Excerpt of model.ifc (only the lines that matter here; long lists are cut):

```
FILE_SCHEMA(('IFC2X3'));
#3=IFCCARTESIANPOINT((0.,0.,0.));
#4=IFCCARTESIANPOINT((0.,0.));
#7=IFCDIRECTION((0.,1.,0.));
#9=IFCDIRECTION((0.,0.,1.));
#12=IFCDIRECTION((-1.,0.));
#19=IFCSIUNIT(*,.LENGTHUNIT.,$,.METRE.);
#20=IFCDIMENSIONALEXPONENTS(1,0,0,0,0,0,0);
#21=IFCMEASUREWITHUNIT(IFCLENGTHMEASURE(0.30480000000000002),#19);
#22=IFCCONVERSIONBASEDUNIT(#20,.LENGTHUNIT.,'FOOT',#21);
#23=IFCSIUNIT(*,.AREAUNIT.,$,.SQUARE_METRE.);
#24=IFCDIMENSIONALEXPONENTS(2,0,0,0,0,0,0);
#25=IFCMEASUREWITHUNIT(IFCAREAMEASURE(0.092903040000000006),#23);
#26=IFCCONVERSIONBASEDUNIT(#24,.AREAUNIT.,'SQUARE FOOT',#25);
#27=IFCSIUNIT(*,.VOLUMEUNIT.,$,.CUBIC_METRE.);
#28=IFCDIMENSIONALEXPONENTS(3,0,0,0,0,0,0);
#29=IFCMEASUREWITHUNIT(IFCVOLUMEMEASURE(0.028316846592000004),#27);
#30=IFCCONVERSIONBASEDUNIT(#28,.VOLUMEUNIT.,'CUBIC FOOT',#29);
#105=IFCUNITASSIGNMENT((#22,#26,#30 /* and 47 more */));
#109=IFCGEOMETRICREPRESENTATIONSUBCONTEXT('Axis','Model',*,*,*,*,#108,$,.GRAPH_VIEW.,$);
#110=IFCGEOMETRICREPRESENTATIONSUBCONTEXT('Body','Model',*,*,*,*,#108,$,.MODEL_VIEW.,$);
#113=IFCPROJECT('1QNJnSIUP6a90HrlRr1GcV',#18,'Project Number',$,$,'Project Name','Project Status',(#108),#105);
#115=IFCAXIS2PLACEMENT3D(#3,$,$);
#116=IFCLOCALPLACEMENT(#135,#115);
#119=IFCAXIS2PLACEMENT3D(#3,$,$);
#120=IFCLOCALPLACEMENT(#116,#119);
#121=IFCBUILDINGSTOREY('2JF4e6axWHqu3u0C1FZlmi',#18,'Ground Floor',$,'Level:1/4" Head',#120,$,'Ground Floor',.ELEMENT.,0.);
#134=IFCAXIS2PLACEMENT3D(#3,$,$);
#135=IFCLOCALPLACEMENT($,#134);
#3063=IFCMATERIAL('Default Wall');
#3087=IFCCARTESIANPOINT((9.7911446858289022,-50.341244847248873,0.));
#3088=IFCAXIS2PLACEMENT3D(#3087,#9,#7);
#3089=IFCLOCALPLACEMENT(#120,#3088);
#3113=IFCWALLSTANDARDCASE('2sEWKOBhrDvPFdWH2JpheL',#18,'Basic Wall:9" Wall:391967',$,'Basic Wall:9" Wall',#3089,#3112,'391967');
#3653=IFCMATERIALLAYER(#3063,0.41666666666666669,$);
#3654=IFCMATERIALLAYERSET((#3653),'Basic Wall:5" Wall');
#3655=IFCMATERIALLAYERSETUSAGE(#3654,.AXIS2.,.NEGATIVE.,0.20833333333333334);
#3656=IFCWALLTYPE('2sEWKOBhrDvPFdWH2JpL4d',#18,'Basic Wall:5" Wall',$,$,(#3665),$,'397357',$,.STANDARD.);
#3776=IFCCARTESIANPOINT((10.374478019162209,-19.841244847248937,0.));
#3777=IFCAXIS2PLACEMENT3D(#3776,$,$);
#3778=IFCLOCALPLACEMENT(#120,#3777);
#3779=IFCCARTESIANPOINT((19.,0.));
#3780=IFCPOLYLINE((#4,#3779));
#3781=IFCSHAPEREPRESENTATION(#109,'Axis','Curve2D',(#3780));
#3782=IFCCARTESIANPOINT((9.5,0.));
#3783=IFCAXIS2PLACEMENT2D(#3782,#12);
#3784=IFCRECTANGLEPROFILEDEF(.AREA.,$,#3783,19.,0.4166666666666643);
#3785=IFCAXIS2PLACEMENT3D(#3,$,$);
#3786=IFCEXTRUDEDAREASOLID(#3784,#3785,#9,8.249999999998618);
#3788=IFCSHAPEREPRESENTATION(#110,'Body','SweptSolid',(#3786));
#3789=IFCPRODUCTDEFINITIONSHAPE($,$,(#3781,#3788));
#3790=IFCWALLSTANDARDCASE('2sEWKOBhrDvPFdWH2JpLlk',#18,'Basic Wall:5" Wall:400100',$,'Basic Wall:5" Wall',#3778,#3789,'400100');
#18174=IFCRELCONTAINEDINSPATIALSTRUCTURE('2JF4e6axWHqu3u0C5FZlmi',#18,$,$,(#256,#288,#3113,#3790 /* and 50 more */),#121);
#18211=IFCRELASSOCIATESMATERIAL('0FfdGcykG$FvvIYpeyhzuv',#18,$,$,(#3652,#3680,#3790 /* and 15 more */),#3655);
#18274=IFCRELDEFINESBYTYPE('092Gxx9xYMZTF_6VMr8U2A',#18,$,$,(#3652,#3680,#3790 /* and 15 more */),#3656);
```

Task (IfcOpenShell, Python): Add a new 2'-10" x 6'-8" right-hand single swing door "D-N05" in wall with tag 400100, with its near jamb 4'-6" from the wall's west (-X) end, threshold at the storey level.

```python
import numpy as np
import ifcopenshell
import ifcopenshell.api.feature
import ifcopenshell.api.geometry
import ifcopenshell.api.root
import ifcopenshell.api.spatial
import ifcopenshell.api.type
import ifcopenshell.geom
import ifcopenshell.util.element
import ifcopenshell.util.placement
import ifcopenshell.util.representation
import ifcopenshell.util.shape
import ifcopenshell.util.unit

model = ifcopenshell.open("model.ifc")
unit_scale = ifcopenshell.util.unit.calculate_unit_scale(model)
settings = ifcopenshell.geom.settings()


def volume(element):
    """Net volume in cubic metres, openings subtracted."""
    shape = ifcopenshell.geom.create_shape(settings, element)
    return ifcopenshell.util.shape.get_volume(shape.geometry)


wall = model.by_guid("2sEWKOBhrDvPFdWH2JpLlk")
storey = ifcopenshell.util.element.get_container(wall, ifc_class="IfcBuildingStorey")
context = ifcopenshell.util.representation.get_context(model, "Model", "Body", "MODEL_VIEW")
before = volume(wall)

width, height, from_end, sill = 0.8636, 2.032, 1.3716, 0.0  # metres

# The wall runs along its own X axis, and the end named is its -X end.
wall_shape = ifcopenshell.geom.create_shape(settings, wall)
x, y, z = ifcopenshell.util.shape.get_vertices(wall_shape.geometry).T
start = x.min() + from_end
face, thickness = float(y.min()), float(y.max() - y.min())
wall_matrix = ifcopenshell.util.placement.get_local_placement(wall.ObjectPlacement)
level = ifcopenshell.util.placement.get_local_placement(storey.ObjectPlacement)[2, 3]


def in_wall(x, y):
    """Placement at x, y metres in the wall's axes, at sill height."""
    matrix = wall_matrix.copy()
    matrix[:, 3] = wall_matrix @ np.array([x / unit_scale, y / unit_scale, 0.0, 1.0])
    matrix[2, 3] = level + sill / unit_scale
    return matrix


# Opening: a box that overshoots both wall faces by 50 mm.
opening = ifcopenshell.api.root.create_entity(model, ifc_class="IfcOpeningElement")
box = ifcopenshell.api.geometry.add_wall_representation(
    model, context=context, length=width, height=height, thickness=thickness + 0.1
)
ifcopenshell.api.geometry.assign_representation(model, product=opening, representation=box)
ifcopenshell.api.geometry.edit_object_placement(model, product=opening, matrix=in_wall(start, face - 0.05), is_si=False)
ifcopenshell.api.feature.add_feature(model, feature=opening, element=wall)

door = ifcopenshell.api.root.create_entity(model, ifc_class="IfcDoor", name="D-N05")
door.OverallWidth, door.OverallHeight = width / unit_scale, height / unit_scale
body = ifcopenshell.api.geometry.add_door_representation(
    model,
    context=context,
    overall_width=door.OverallWidth,
    overall_height=door.OverallHeight,
    operation_type="SINGLE_SWING_RIGHT",
    lining_properties={"LiningDepth": thickness / unit_scale, "ThresholdDepth": thickness / unit_scale},
)
ifcopenshell.api.geometry.assign_representation(model, product=door, representation=body)
ifcopenshell.api.spatial.assign_container(model, products=[door], relating_structure=storey)
fills = ifcopenshell.api.feature.add_filling(model, opening=opening, element=door)
fills.OwnerHistory = door.OwnerHistory  # required in IFC2X3

# IFC2X3 keeps the operation on the door style.
style = ifcopenshell.api.root.create_entity(model, ifc_class="IfcDoorStyle", name="D-N05")
style.OperationType, style.ConstructionType = "SINGLE_SWING_RIGHT", "NOTDEFINED"
style.ParameterTakesPrecedence = style.Sizeable = False
ifcopenshell.api.type.assign_type(model, related_objects=[door], relating_type=style)

# The lining spans the wall, so the door starts at the wall face.
ifcopenshell.api.geometry.edit_object_placement(model, product=door, matrix=in_wall(start, face), is_si=False)

after = volume(wall)

print(f"wall volume {before:.3f} -> {after:.3f} m3")

model.write("model_rev.ifc")
```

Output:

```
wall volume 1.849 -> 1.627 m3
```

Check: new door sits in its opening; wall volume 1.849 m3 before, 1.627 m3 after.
